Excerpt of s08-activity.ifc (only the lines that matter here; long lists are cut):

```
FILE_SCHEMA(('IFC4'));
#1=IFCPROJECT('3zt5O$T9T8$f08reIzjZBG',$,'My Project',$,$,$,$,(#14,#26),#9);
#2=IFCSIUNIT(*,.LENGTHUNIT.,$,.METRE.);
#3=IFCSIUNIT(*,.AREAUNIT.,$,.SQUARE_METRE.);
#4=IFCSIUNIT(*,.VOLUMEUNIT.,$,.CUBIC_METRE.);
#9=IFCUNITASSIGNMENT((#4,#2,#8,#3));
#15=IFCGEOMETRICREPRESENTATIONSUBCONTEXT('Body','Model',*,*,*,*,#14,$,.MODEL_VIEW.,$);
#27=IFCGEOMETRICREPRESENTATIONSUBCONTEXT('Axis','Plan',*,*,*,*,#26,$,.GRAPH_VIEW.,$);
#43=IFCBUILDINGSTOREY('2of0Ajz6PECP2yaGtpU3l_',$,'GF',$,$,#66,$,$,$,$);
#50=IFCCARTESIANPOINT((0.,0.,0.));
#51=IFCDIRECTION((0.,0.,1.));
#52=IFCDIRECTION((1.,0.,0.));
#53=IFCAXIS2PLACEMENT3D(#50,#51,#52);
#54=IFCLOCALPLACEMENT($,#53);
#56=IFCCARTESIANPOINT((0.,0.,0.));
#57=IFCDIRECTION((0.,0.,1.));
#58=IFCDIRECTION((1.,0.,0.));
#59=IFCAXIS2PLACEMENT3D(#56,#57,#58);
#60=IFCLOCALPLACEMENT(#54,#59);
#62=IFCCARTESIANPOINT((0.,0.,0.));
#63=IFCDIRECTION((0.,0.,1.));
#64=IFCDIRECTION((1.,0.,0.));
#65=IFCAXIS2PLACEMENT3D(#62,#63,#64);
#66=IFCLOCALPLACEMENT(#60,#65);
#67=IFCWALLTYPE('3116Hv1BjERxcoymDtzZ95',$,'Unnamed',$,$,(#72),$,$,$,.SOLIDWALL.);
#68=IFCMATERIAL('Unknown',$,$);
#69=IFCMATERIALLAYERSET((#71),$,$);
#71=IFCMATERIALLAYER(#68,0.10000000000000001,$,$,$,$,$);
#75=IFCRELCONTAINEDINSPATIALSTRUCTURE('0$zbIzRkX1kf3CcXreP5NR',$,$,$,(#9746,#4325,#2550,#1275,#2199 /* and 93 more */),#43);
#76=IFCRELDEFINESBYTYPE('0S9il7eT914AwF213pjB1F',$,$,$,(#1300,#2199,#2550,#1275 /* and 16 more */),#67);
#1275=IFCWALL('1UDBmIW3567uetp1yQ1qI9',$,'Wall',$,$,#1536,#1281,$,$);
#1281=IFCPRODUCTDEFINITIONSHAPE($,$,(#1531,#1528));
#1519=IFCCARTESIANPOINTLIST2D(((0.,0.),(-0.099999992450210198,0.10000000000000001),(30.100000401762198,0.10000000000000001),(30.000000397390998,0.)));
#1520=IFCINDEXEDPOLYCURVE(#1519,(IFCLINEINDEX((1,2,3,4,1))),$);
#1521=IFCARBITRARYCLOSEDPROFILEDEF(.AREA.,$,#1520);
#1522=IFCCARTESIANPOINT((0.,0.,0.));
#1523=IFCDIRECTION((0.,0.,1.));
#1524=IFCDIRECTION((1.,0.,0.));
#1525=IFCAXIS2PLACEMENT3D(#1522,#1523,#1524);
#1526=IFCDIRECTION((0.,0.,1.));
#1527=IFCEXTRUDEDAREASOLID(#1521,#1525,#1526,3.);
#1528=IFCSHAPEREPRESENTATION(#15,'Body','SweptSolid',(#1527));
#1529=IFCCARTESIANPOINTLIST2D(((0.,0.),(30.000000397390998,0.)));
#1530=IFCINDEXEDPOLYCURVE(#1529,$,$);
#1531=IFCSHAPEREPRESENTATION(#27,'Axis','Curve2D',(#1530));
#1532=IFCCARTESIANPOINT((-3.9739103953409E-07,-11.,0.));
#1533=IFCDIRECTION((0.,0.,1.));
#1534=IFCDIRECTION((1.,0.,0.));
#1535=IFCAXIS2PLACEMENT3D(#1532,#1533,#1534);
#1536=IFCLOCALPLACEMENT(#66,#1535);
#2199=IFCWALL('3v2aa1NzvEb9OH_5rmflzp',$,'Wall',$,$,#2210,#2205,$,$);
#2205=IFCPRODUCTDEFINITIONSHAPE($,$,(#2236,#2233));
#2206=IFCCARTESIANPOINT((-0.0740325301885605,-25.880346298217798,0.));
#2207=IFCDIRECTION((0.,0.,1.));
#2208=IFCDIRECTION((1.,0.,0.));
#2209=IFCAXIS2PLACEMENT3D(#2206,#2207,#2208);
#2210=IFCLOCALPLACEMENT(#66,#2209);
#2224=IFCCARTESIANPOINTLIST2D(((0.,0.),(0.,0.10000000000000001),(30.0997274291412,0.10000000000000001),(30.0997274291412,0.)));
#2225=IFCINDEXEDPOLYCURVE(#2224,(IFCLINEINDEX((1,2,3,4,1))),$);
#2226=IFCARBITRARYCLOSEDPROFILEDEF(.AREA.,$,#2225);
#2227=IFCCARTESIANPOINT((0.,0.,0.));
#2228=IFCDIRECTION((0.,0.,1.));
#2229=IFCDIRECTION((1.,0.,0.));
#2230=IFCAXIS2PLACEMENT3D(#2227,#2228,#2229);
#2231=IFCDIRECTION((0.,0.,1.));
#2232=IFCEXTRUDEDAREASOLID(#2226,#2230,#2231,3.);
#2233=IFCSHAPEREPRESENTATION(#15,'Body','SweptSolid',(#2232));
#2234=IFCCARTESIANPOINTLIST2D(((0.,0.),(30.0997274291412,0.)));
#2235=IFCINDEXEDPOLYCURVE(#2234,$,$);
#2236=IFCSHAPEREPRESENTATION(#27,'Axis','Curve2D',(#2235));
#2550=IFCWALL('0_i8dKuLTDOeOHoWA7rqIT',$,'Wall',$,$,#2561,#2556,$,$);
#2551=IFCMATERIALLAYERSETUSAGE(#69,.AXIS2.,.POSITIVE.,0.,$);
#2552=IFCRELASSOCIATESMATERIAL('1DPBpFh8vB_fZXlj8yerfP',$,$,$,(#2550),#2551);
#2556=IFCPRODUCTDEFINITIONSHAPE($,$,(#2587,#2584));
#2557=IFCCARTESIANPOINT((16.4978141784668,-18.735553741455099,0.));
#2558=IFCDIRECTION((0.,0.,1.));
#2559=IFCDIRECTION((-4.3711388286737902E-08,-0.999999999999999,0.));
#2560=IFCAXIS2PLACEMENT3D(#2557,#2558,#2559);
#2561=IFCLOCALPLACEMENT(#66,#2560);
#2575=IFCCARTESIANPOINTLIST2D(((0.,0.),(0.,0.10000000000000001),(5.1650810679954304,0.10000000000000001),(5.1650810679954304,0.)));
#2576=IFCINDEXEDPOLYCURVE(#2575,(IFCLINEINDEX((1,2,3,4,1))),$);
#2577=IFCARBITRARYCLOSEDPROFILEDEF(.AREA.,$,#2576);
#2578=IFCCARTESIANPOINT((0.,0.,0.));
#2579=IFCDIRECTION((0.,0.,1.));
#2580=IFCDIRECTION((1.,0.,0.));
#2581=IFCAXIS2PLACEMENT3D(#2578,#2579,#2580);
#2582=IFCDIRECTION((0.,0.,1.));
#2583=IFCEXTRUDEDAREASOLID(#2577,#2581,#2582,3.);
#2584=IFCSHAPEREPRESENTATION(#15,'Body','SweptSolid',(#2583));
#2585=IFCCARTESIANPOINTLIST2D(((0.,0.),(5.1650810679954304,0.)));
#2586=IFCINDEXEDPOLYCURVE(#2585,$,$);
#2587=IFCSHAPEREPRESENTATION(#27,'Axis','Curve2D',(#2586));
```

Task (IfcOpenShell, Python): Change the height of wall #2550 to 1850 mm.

```python
import ifcopenshell
import ifcopenshell.geom
import ifcopenshell.util.representation
import ifcopenshell.util.shape
import ifcopenshell.util.unit

model = ifcopenshell.open("s08-activity.ifc")
unit_scale = ifcopenshell.util.unit.calculate_unit_scale(model)
settings = ifcopenshell.geom.settings()


def volume(element):
    """Net volume in cubic metres, openings subtracted."""
    shape = ifcopenshell.geom.create_shape(settings, element)
    return ifcopenshell.util.shape.get_volume(shape.geometry)


wall = model.by_guid("0_i8dKuLTDOeOHoWA7rqIT")
before = volume(wall)

body = ifcopenshell.util.representation.get_representation(wall, "Model", "Body")
solid = body.Items[0]
old_height = solid.Depth
solid.Depth = 1.85 / unit_scale
after = volume(wall)

print(f"height {old_height:g} -> {solid.Depth:g}, volume {before:.3f} -> {after:.3f} m3")

model.write("s08-activity_updated.ifc")
```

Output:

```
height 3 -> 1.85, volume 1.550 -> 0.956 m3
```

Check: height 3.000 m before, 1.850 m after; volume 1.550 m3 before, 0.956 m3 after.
